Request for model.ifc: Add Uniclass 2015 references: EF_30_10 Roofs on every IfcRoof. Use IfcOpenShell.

First a look at what the model holds.

```python
import ifcopenshell

model = ifcopenshell.open("model.ifc")
print(model.schema)
print("classifications:", [c.Name for c in model.by_type("IfcClassification")])
for ifc_class in ("IfcDoor", "IfcRoof", "IfcStair", "IfcWall", "IfcWindow"):
    print(ifc_class, len(model.by_type(ifc_class)))
```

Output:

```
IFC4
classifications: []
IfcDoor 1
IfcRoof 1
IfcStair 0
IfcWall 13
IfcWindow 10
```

```python
import ifcopenshell
import ifcopenshell.api.classification

model = ifcopenshell.open("model.ifc")

system = ifcopenshell.api.classification.add_classification(model, classification="Uniclass 2015")

codes = {
    "IfcRoof": ("EF_30_10", "Roofs"),
}
for ifc_class, (code, name) in codes.items():
    products = model.by_type(ifc_class)
    ifcopenshell.api.classification.add_reference(
        model, products=products, classification=system, identification=code, name=name
    )
    print(code, len(products))

model.write("model_edited.ifc")
```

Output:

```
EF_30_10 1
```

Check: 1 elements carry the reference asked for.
